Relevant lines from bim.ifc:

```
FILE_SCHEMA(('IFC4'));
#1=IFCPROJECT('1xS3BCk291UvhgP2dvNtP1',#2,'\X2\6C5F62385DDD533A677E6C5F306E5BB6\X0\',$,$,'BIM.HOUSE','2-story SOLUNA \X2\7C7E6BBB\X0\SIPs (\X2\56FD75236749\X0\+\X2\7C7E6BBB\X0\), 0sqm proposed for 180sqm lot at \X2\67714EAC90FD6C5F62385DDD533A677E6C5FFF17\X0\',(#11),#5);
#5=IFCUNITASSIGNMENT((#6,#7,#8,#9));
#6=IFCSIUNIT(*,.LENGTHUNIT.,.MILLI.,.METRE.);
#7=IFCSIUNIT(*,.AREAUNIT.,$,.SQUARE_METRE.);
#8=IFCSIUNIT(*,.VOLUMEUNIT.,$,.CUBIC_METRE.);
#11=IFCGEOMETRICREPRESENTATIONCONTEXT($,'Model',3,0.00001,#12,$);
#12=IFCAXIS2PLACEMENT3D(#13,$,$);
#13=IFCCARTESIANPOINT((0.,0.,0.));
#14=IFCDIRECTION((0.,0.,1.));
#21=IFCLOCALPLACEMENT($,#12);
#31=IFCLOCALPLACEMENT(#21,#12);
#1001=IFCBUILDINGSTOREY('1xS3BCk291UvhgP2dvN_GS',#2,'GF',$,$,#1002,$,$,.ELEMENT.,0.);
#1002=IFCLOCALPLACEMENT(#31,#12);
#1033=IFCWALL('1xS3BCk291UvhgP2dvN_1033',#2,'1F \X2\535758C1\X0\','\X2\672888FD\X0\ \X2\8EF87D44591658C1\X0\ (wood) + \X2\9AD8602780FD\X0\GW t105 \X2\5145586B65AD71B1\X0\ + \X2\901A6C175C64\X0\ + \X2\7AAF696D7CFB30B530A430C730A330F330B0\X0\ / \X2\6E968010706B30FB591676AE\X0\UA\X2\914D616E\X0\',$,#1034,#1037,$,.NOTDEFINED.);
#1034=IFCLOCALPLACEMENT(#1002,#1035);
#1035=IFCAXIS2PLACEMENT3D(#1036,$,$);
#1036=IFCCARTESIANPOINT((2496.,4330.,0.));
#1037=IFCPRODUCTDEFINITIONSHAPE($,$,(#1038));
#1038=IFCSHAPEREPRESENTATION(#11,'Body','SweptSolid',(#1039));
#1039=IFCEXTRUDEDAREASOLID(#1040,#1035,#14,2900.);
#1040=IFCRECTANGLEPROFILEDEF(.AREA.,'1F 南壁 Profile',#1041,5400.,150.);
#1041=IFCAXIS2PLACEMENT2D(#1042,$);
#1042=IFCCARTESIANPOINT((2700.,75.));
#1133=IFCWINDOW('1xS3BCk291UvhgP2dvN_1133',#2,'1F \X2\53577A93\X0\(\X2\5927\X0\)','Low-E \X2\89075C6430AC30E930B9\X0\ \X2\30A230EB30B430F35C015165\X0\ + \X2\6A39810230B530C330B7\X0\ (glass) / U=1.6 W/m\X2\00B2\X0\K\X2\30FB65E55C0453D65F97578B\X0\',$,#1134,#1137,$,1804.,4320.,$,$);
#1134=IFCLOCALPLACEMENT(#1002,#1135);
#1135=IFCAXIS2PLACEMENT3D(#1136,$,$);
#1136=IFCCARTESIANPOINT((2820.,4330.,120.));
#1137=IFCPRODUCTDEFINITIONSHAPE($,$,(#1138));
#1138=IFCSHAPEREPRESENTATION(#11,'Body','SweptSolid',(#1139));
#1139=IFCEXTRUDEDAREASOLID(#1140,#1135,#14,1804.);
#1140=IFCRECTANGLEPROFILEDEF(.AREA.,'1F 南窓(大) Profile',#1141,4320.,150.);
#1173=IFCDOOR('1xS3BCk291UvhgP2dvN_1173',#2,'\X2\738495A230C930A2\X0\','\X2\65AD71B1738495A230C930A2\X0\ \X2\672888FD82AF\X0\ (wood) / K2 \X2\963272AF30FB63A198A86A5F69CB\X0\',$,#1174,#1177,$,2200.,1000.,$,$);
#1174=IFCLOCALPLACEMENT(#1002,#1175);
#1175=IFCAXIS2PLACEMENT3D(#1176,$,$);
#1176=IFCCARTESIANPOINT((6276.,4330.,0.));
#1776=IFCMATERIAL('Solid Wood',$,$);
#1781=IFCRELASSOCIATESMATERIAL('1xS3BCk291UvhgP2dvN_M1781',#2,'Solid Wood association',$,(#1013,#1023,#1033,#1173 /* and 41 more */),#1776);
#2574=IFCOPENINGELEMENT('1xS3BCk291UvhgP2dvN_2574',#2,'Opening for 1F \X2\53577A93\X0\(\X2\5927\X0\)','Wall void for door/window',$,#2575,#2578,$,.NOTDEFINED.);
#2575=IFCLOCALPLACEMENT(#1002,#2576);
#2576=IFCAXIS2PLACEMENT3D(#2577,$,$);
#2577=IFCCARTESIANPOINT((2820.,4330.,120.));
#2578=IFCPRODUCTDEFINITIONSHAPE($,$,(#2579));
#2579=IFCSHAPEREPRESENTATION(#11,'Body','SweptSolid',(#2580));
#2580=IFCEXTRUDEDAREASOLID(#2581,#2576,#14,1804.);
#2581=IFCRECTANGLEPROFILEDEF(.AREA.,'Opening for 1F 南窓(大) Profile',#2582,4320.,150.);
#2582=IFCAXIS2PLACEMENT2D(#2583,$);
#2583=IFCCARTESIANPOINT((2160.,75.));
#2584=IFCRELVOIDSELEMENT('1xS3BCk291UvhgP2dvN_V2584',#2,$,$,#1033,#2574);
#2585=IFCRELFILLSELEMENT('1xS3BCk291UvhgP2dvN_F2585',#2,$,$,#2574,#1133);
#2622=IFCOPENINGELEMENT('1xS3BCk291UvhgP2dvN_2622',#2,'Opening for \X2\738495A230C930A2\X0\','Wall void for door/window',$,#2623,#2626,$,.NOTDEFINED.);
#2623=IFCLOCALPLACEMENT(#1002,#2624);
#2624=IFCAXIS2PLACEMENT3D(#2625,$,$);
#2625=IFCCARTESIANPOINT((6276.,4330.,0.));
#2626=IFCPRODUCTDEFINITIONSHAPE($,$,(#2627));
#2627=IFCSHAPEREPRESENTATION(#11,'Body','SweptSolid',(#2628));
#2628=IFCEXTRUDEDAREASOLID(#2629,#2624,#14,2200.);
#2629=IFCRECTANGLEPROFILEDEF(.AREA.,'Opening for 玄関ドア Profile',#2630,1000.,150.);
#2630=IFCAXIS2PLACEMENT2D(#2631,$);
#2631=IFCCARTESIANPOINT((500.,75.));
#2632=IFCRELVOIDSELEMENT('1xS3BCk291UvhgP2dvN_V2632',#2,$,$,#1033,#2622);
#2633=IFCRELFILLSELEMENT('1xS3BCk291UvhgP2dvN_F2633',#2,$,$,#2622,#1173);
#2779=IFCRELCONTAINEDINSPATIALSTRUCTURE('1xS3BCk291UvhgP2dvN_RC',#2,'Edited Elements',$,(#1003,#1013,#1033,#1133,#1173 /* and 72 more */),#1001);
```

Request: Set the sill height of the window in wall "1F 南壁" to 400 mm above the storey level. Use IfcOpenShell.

```python
import numpy as np
import ifcopenshell
import ifcopenshell.api.geometry
import ifcopenshell.geom
import ifcopenshell.util.element
import ifcopenshell.util.placement
import ifcopenshell.util.shape
import ifcopenshell.util.unit

model = ifcopenshell.open("bim.ifc")
unit_scale = ifcopenshell.util.unit.calculate_unit_scale(model)

window = model.by_guid("1xS3BCk291UvhgP2dvN_1133")
opening = window.FillsVoids[0].RelatingOpeningElement
storey = ifcopenshell.util.element.get_container(window, ifc_class="IfcBuildingStorey")
level = ifcopenshell.util.placement.get_local_placement(storey.ObjectPlacement)[2, 3]

# The opening's origin need not be at the sill, so measure its lowest point.
shape = ifcopenshell.geom.create_shape(ifcopenshell.geom.settings(), opening)
bottom = ifcopenshell.util.shape.get_shape_bottom_elevation(shape, shape.geometry) / unit_scale
dz = level + 0.4 / unit_scale - bottom

shift = np.array([0.0, 0.0, dz])
# The window is not placed relative to its opening, so move both.
for product in (opening, window):
    matrix = ifcopenshell.util.placement.get_local_placement(product.ObjectPlacement)
    matrix[:3, 3] += shift
    ifcopenshell.api.geometry.edit_object_placement(model, product=product, matrix=matrix, is_si=False)

print(f"moved by {dz * unit_scale:+.3f} m")

model.write("bim-out.ifc")
```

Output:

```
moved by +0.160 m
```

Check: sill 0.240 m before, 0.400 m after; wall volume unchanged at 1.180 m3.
